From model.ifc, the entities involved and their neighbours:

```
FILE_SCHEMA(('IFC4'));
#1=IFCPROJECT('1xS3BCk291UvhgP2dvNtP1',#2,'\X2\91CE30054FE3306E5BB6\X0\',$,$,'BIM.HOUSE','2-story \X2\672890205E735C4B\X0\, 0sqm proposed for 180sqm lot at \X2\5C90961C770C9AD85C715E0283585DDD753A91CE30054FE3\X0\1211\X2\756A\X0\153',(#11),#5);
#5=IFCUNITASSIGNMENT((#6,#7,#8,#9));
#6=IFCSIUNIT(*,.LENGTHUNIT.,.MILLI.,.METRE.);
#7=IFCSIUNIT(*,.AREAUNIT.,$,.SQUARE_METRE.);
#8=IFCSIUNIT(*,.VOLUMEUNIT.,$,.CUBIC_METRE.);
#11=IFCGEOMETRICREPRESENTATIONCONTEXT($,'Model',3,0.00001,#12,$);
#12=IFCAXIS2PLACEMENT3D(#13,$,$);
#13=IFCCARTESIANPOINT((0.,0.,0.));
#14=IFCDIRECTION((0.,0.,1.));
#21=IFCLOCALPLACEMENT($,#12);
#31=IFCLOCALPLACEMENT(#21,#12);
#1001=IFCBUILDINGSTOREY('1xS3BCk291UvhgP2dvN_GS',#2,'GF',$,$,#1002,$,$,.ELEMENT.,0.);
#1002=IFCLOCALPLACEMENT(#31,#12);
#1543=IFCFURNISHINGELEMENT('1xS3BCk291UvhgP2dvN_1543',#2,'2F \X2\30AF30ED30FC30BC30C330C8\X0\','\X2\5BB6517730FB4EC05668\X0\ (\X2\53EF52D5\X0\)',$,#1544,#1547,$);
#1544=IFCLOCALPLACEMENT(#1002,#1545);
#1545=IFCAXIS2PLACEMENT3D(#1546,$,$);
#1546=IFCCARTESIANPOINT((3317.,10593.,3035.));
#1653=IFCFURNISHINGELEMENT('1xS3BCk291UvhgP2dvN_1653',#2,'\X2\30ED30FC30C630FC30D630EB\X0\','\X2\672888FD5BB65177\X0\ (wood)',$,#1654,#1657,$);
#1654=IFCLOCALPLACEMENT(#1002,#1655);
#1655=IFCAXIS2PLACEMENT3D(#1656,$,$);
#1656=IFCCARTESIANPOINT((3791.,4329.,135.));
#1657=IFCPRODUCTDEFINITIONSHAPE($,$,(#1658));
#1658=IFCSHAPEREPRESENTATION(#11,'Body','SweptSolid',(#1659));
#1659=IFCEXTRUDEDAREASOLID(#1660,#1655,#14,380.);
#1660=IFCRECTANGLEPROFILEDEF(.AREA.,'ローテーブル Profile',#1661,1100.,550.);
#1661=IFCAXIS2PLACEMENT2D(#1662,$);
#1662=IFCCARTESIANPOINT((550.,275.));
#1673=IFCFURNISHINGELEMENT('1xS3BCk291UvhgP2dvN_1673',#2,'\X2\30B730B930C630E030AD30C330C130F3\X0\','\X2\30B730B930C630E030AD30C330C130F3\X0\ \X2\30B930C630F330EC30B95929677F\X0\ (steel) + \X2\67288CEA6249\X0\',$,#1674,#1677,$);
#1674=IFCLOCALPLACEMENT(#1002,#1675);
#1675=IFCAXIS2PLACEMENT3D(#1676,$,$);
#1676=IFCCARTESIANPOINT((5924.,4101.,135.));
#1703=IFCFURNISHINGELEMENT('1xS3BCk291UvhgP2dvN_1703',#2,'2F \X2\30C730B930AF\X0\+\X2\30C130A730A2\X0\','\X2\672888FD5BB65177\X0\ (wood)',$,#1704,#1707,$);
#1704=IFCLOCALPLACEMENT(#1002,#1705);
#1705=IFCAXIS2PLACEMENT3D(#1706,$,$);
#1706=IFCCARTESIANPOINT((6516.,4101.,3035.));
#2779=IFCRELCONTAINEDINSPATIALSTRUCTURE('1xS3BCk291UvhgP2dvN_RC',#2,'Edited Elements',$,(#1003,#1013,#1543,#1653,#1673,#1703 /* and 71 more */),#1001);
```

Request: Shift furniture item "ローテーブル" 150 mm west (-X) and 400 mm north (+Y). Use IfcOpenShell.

```python
import ifcopenshell
import ifcopenshell.api.geometry
import ifcopenshell.util.placement

model = ifcopenshell.open("model.ifc")

item = model.by_guid("1xS3BCk291UvhgP2dvN_1653")
matrix = ifcopenshell.util.placement.get_local_placement(item.ObjectPlacement)
matrix[0, 3] -= 150.0
matrix[1, 3] += 400.0
ifcopenshell.api.geometry.edit_object_placement(model, product=item, matrix=matrix, is_si=False)

print(ifcopenshell.util.placement.get_local_placement(item.ObjectPlacement).round(3) + 0.0)

model.write("model_edited.ifc")
```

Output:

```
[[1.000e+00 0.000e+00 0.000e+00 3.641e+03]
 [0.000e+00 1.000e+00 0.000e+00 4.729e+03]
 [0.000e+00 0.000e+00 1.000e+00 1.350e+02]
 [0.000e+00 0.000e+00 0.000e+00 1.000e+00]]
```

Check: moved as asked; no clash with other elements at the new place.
